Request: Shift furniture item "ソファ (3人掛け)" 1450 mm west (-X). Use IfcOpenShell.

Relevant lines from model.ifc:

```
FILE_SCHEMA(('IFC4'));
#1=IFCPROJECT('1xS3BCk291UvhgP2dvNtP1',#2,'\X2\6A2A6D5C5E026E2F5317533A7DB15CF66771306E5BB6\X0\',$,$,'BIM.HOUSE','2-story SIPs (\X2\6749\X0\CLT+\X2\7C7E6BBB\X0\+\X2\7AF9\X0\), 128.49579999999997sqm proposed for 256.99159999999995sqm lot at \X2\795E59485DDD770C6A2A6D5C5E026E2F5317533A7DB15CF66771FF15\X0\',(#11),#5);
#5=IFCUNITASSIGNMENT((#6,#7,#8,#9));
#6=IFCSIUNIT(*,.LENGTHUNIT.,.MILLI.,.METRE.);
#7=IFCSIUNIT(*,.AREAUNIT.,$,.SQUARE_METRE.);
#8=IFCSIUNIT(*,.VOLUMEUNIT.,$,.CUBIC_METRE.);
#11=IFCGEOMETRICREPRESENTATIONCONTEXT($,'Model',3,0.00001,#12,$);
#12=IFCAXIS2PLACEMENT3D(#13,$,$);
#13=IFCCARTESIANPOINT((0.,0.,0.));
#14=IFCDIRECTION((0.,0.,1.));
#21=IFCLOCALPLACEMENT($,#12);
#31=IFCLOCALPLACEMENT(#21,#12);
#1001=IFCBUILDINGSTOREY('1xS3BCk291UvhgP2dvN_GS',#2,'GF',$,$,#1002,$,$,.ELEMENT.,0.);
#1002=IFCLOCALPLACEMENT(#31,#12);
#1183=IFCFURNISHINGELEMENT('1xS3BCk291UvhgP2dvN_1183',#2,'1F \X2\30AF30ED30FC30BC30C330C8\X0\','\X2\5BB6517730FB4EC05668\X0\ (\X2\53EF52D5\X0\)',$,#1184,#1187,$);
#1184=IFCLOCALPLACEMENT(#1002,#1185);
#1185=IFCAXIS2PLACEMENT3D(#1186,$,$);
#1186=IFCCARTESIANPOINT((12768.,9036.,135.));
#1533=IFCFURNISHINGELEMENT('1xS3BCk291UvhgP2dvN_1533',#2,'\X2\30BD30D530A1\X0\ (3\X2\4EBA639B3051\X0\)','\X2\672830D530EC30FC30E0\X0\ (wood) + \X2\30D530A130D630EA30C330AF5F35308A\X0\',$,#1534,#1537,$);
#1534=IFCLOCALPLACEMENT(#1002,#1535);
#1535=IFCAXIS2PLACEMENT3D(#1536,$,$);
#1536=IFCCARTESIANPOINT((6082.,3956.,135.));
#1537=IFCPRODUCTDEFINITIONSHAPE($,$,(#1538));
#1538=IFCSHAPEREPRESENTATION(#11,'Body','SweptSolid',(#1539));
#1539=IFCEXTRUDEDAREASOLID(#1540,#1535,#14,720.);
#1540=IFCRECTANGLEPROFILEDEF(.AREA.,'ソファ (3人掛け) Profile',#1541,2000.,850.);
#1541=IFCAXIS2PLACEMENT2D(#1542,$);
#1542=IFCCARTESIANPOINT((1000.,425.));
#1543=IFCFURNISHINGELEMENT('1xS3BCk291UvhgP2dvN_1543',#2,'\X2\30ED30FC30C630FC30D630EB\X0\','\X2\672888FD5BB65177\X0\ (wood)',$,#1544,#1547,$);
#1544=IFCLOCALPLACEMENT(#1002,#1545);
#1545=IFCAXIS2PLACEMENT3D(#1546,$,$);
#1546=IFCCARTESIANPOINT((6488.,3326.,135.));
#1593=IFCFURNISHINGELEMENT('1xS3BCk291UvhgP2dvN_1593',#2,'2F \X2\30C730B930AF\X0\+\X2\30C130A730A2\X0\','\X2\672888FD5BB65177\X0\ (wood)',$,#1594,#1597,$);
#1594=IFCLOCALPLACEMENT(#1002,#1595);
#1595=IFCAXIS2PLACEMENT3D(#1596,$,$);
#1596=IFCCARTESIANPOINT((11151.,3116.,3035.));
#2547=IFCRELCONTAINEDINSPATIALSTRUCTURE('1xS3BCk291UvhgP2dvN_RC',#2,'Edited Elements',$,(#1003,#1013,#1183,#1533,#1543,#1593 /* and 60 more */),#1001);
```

```python
import ifcopenshell
import ifcopenshell.api.geometry
import ifcopenshell.util.placement
import ifcopenshell.util.unit

model = ifcopenshell.open("model.ifc")
unit_scale = ifcopenshell.util.unit.calculate_unit_scale(model)

item = model.by_guid("1xS3BCk291UvhgP2dvN_1533")
matrix = ifcopenshell.util.placement.get_local_placement(item.ObjectPlacement)
matrix[0, 3] -= 1.45 / unit_scale
ifcopenshell.api.geometry.edit_object_placement(model, product=item, matrix=matrix, is_si=False)

print(ifcopenshell.util.placement.get_local_placement(item.ObjectPlacement).round(3) + 0.0)

model.write("model_updated.ifc")
```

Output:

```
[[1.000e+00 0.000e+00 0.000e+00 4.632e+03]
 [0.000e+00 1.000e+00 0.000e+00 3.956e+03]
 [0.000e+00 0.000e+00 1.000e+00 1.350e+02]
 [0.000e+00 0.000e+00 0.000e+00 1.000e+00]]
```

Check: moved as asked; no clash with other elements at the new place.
